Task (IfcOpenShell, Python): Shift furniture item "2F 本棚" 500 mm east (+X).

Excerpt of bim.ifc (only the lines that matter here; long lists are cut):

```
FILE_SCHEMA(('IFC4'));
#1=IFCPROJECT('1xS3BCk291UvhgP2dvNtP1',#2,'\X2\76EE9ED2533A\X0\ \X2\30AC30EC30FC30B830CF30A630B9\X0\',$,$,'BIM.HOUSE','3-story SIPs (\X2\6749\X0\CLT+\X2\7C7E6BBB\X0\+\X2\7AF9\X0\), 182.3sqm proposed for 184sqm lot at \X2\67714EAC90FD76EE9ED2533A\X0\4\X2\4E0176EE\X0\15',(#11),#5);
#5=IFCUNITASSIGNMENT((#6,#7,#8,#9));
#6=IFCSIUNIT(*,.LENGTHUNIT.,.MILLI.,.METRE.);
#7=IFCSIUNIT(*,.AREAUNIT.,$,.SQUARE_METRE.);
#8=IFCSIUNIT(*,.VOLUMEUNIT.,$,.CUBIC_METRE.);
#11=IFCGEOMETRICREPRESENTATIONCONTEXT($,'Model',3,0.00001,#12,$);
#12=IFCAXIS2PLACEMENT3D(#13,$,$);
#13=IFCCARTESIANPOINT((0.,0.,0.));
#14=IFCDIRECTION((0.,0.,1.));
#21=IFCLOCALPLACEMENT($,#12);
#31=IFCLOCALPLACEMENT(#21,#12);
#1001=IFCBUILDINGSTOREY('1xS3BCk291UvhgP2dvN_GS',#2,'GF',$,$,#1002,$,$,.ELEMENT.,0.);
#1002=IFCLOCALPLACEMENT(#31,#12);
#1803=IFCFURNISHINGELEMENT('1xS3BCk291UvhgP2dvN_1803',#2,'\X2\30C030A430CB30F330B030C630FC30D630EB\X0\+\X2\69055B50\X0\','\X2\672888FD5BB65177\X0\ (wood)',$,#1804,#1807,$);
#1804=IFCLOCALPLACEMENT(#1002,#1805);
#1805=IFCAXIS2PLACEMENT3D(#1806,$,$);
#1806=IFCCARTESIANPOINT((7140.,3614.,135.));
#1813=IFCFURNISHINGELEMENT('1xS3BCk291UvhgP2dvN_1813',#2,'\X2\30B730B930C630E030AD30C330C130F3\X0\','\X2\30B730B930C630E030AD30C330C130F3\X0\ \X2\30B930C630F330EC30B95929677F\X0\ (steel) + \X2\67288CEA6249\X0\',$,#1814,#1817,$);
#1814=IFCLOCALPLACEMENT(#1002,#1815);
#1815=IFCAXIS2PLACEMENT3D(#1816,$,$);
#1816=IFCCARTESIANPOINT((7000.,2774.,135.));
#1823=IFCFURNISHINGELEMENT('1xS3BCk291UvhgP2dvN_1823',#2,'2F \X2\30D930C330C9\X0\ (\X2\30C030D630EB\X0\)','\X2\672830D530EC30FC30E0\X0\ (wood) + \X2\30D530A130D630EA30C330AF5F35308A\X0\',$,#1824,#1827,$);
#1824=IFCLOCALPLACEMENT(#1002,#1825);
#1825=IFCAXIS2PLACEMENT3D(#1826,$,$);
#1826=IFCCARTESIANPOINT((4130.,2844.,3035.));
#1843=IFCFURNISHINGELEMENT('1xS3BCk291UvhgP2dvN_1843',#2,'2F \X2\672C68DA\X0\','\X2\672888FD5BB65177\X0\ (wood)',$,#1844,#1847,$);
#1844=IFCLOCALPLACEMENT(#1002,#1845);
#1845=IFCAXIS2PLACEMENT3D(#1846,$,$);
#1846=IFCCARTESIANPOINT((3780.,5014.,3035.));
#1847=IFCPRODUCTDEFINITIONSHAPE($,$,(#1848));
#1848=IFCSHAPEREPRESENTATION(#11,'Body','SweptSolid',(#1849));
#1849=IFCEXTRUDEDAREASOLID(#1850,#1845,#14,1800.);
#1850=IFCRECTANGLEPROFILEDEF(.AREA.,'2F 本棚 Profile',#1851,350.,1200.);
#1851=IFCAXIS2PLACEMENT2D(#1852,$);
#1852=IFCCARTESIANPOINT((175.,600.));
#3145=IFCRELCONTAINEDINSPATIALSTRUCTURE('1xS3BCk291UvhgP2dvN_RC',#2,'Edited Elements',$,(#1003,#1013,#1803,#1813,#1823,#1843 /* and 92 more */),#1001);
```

```python
import ifcopenshell
import ifcopenshell.api.geometry
import ifcopenshell.util.placement
import ifcopenshell.util.unit

model = ifcopenshell.open("bim.ifc")
unit_scale = ifcopenshell.util.unit.calculate_unit_scale(model)

item = model.by_id(1843)
matrix = ifcopenshell.util.placement.get_local_placement(item.ObjectPlacement)
matrix[0, 3] += 0.5 / unit_scale
ifcopenshell.api.geometry.edit_object_placement(model, product=item, matrix=matrix, is_si=False)

print(ifcopenshell.util.placement.get_local_placement(item.ObjectPlacement).round(3) + 0.0)

model.write("bim-out.ifc")
```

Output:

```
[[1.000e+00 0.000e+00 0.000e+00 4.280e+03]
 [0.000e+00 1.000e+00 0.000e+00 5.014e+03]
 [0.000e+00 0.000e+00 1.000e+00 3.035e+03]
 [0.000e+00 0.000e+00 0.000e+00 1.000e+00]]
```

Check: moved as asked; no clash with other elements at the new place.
